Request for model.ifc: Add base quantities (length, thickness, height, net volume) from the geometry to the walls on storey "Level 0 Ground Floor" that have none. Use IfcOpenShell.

First a look at what the model holds.

```python
import ifcopenshell
import ifcopenshell.util.element
import ifcopenshell.util.unit

model = ifcopenshell.open("model.ifc")
print(model.schema)
for unit_type in ("LENGTHUNIT", "AREAUNIT", "VOLUMEUNIT"):
    print(unit_type, ifcopenshell.util.unit.calculate_unit_scale(model, unit_type))
storey = next(s for s in model.by_type("IfcBuildingStorey") if s.Name == "Level 0 Ground Floor")
walls = [e for e in ifcopenshell.util.element.get_decomposition(storey) if e.is_a("IfcWall")]
for e in sorted(walls, key=lambda e: e.id()):
    print(e.id(), e.is_a(), e.Name, list(ifcopenshell.util.element.get_psets(e, qtos_only=True)), sep=" | ")
```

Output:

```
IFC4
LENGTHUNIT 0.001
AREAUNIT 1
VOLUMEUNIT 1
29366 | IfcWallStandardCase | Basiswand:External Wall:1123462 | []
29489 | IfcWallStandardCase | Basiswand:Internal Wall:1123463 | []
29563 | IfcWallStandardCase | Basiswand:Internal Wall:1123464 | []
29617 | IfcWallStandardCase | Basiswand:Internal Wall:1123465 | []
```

```python
import ifcopenshell
import ifcopenshell.api.pset
import ifcopenshell.geom
import ifcopenshell.util.element
import ifcopenshell.util.shape
import ifcopenshell.util.unit

model = ifcopenshell.open("model.ifc")
unit_scale = ifcopenshell.util.unit.calculate_unit_scale(model)
volume_scale = ifcopenshell.util.unit.calculate_unit_scale(model, "VOLUMEUNIT")
settings = ifcopenshell.geom.settings()

storey = next(s for s in model.by_type("IfcBuildingStorey") if s.Name == "Level 0 Ground Floor")
walls = [e for e in ifcopenshell.util.element.get_decomposition(storey) if e.is_a("IfcWall")]

for e in sorted(walls, key=lambda e: e.id()):
    if ifcopenshell.util.element.get_psets(e, qtos_only=True, should_inherit=False):
        continue
    # Geometry comes back in metres, in the element's own axes.
    shape = ifcopenshell.geom.create_shape(settings, e)
    values = {
        "Length": ifcopenshell.util.shape.get_x(shape.geometry) / unit_scale,
        "Width": ifcopenshell.util.shape.get_y(shape.geometry) / unit_scale,
        "Height": ifcopenshell.util.shape.get_z(shape.geometry) / unit_scale,
        "NetVolume": ifcopenshell.util.shape.get_volume(shape.geometry) / volume_scale,
    }
    qto = ifcopenshell.api.pset.add_qto(model, product=e, name="Qto_WallBaseQuantities")
    ifcopenshell.api.pset.edit_qto(model, qto=qto, properties=values)
    print(e.id(), {k: round(v, 3) for k, v in values.items()})

model.write("model_updated.ifc")
```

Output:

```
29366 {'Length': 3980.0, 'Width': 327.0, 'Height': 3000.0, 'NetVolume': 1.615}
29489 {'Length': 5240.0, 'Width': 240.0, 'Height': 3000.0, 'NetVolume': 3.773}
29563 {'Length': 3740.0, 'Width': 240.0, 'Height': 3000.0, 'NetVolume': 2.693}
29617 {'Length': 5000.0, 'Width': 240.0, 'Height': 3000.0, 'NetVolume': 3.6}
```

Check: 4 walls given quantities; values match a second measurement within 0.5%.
